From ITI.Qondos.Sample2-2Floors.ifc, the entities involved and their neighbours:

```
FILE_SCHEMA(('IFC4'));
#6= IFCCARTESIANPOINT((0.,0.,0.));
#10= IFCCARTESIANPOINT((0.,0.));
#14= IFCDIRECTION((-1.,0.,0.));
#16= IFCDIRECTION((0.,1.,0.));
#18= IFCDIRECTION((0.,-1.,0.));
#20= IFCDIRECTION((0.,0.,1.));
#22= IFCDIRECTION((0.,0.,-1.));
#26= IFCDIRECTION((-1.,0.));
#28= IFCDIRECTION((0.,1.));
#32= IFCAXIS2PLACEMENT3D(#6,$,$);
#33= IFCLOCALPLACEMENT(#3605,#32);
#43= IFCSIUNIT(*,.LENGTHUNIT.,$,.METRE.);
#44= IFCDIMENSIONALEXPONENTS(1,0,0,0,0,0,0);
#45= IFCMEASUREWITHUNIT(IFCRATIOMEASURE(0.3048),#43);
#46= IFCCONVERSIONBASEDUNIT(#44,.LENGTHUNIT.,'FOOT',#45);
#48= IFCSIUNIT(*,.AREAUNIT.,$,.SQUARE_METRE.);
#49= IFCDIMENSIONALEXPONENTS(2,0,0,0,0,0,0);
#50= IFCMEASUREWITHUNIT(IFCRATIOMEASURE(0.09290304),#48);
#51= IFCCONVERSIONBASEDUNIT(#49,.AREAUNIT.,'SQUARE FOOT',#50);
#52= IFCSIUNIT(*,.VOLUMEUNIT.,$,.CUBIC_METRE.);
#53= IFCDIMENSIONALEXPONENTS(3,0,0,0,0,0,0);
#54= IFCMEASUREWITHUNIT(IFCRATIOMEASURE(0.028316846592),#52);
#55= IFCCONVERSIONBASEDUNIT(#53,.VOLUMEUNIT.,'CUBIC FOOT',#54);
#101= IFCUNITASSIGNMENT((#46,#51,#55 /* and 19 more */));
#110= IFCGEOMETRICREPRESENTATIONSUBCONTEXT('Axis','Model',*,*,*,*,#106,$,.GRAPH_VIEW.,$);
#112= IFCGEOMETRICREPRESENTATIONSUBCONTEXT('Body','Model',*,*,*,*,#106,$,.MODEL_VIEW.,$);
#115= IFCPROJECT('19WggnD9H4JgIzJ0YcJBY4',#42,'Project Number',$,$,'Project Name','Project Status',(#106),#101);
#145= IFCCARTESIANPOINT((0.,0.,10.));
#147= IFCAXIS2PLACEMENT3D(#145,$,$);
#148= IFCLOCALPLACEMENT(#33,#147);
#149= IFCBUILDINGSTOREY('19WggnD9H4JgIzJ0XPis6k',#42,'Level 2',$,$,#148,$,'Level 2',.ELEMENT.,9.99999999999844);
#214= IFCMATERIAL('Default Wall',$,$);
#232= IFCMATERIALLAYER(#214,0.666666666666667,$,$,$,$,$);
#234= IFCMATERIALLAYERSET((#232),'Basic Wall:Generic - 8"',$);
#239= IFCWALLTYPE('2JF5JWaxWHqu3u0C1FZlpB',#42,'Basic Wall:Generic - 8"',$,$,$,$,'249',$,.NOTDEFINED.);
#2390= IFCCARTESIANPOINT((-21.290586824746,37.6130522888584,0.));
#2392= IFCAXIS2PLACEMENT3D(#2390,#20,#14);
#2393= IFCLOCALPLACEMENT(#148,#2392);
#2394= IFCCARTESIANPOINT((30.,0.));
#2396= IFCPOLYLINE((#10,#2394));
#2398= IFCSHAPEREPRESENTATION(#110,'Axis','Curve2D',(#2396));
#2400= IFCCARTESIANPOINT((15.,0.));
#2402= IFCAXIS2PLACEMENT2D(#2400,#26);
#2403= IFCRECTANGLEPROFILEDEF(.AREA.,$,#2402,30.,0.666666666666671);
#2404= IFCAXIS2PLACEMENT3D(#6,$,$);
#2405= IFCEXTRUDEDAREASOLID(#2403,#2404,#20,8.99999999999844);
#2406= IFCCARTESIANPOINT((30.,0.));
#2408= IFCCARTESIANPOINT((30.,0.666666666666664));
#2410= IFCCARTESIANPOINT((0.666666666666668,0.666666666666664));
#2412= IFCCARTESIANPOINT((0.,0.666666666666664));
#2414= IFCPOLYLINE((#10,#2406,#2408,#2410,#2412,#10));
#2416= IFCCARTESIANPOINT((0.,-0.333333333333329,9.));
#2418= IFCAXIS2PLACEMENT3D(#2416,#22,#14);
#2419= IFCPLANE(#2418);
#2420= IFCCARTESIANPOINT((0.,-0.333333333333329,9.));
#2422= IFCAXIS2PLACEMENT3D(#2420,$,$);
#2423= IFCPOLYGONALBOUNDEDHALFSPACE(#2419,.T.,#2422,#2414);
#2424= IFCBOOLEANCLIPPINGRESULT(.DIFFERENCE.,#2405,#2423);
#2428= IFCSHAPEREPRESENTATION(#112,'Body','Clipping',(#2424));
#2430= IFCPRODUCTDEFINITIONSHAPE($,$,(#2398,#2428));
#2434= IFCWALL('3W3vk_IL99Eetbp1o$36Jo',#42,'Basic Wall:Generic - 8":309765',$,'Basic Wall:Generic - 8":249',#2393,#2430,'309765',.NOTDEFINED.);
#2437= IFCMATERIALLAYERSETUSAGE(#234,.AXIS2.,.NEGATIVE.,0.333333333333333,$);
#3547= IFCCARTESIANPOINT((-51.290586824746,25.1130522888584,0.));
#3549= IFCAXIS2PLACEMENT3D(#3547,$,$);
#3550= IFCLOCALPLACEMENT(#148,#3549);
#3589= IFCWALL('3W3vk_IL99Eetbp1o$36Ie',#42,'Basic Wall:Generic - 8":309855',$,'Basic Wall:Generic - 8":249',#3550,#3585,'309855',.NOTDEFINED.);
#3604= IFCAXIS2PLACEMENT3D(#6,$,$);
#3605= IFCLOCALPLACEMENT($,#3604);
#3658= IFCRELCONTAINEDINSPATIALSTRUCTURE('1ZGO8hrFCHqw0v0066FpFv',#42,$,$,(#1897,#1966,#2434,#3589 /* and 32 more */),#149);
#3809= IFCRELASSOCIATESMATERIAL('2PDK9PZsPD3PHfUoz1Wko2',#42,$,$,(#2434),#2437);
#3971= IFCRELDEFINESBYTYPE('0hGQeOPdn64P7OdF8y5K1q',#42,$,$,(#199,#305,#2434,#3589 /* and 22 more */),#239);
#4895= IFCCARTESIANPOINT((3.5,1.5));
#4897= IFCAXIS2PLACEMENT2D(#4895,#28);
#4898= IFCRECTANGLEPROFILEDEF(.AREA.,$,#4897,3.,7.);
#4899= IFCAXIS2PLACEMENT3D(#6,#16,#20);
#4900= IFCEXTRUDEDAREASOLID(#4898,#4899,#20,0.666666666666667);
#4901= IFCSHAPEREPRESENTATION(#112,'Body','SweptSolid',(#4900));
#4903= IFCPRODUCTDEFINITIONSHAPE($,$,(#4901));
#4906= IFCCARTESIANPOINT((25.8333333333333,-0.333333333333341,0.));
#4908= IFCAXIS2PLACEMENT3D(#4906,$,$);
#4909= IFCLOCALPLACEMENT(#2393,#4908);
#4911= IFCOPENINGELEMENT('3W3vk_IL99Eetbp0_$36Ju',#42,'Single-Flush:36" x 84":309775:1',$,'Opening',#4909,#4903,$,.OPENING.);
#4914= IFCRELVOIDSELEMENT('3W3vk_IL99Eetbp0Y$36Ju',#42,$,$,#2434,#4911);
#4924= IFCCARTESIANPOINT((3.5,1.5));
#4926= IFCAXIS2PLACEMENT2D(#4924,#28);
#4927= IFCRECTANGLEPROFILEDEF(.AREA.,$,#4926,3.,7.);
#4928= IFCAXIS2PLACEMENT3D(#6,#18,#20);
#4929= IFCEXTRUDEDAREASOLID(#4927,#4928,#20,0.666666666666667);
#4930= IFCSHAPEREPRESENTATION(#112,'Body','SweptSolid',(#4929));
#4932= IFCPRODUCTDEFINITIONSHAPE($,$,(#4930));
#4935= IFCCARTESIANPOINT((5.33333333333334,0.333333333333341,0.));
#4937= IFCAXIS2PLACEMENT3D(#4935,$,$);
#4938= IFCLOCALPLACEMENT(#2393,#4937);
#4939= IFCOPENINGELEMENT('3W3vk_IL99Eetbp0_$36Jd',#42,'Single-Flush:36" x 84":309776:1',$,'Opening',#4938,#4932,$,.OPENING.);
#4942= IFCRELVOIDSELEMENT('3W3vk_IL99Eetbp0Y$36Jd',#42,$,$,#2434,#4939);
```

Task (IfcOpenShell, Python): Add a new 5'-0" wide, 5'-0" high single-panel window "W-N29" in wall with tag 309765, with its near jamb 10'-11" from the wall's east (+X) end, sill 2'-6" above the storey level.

```python
import numpy as np
import ifcopenshell
import ifcopenshell.api.feature
import ifcopenshell.api.geometry
import ifcopenshell.api.root
import ifcopenshell.api.spatial
import ifcopenshell.geom
import ifcopenshell.util.element
import ifcopenshell.util.placement
import ifcopenshell.util.representation
import ifcopenshell.util.shape
import ifcopenshell.util.unit

model = ifcopenshell.open("ITI.Qondos.Sample2-2Floors.ifc")
unit_scale = ifcopenshell.util.unit.calculate_unit_scale(model)
settings = ifcopenshell.geom.settings()


def volume(element):
    """Net volume in cubic metres, openings subtracted."""
    shape = ifcopenshell.geom.create_shape(settings, element)
    return ifcopenshell.util.shape.get_volume(shape.geometry)


wall = model.by_guid("3W3vk_IL99Eetbp1o$36Jo")
storey = ifcopenshell.util.element.get_container(wall, ifc_class="IfcBuildingStorey")
context = ifcopenshell.util.representation.get_context(model, "Model", "Body", "MODEL_VIEW")
before = volume(wall)

width, height, from_end, sill = 1.524, 1.524, 3.3274, 0.762  # metres

# The wall runs along its own X axis, and the end named is its -X end.
wall_shape = ifcopenshell.geom.create_shape(settings, wall)
x, y, z = ifcopenshell.util.shape.get_vertices(wall_shape.geometry).T
start = x.min() + from_end
face, thickness = float(y.min()), float(y.max() - y.min())
wall_matrix = ifcopenshell.util.placement.get_local_placement(wall.ObjectPlacement)
level = ifcopenshell.util.placement.get_local_placement(storey.ObjectPlacement)[2, 3]


def in_wall(x, y):
    """Placement at x, y metres in the wall's axes, at sill height."""
    matrix = wall_matrix.copy()
    matrix[:, 3] = wall_matrix @ np.array([x / unit_scale, y / unit_scale, 0.0, 1.0])
    matrix[2, 3] = level + sill / unit_scale
    return matrix


# Opening: a box that overshoots both wall faces by 50 mm.
opening = ifcopenshell.api.root.create_entity(model, ifc_class="IfcOpeningElement", predefined_type="OPENING")
box = ifcopenshell.api.geometry.add_wall_representation(
    model, context=context, length=width, height=height, thickness=thickness + 0.1
)
ifcopenshell.api.geometry.assign_representation(model, product=opening, representation=box)
ifcopenshell.api.geometry.edit_object_placement(model, product=opening, matrix=in_wall(start, face - 0.05), is_si=False)
ifcopenshell.api.feature.add_feature(model, feature=opening, element=wall)

window = ifcopenshell.api.root.create_entity(model, ifc_class="IfcWindow", name="W-N29", predefined_type="WINDOW")
window.OverallWidth, window.OverallHeight = width / unit_scale, height / unit_scale
window.PartitioningType = "SINGLE_PANEL"
body = ifcopenshell.api.geometry.add_window_representation(
    model,
    context=context,
    overall_width=window.OverallWidth,
    overall_height=window.OverallHeight,
    partition_type="SINGLE_PANEL",
)
ifcopenshell.api.geometry.assign_representation(model, product=window, representation=body)
ifcopenshell.api.spatial.assign_container(model, products=[window], relating_structure=storey)
ifcopenshell.api.feature.add_filling(model, opening=opening, element=window)

# Centre the window in the wall's thickness.
ifcopenshell.api.geometry.edit_object_placement(model, product=window, matrix=in_wall(start, face), is_si=False)
window_shape = ifcopenshell.geom.create_shape(settings, window)
depth = ifcopenshell.util.shape.get_vertices(window_shape.geometry)[:, 1]
offset = face + thickness / 2 - (depth.min() + depth.max()) / 2
ifcopenshell.api.geometry.edit_object_placement(model, product=window, matrix=in_wall(start, offset), is_si=False)

after = volume(wall)

print(f"wall volume {before:.3f} -> {after:.3f} m3")

model.write("ITI.Qondos.Sample2-2Floors_v2.ifc")
```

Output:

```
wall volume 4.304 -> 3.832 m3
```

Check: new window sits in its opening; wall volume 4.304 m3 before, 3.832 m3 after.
